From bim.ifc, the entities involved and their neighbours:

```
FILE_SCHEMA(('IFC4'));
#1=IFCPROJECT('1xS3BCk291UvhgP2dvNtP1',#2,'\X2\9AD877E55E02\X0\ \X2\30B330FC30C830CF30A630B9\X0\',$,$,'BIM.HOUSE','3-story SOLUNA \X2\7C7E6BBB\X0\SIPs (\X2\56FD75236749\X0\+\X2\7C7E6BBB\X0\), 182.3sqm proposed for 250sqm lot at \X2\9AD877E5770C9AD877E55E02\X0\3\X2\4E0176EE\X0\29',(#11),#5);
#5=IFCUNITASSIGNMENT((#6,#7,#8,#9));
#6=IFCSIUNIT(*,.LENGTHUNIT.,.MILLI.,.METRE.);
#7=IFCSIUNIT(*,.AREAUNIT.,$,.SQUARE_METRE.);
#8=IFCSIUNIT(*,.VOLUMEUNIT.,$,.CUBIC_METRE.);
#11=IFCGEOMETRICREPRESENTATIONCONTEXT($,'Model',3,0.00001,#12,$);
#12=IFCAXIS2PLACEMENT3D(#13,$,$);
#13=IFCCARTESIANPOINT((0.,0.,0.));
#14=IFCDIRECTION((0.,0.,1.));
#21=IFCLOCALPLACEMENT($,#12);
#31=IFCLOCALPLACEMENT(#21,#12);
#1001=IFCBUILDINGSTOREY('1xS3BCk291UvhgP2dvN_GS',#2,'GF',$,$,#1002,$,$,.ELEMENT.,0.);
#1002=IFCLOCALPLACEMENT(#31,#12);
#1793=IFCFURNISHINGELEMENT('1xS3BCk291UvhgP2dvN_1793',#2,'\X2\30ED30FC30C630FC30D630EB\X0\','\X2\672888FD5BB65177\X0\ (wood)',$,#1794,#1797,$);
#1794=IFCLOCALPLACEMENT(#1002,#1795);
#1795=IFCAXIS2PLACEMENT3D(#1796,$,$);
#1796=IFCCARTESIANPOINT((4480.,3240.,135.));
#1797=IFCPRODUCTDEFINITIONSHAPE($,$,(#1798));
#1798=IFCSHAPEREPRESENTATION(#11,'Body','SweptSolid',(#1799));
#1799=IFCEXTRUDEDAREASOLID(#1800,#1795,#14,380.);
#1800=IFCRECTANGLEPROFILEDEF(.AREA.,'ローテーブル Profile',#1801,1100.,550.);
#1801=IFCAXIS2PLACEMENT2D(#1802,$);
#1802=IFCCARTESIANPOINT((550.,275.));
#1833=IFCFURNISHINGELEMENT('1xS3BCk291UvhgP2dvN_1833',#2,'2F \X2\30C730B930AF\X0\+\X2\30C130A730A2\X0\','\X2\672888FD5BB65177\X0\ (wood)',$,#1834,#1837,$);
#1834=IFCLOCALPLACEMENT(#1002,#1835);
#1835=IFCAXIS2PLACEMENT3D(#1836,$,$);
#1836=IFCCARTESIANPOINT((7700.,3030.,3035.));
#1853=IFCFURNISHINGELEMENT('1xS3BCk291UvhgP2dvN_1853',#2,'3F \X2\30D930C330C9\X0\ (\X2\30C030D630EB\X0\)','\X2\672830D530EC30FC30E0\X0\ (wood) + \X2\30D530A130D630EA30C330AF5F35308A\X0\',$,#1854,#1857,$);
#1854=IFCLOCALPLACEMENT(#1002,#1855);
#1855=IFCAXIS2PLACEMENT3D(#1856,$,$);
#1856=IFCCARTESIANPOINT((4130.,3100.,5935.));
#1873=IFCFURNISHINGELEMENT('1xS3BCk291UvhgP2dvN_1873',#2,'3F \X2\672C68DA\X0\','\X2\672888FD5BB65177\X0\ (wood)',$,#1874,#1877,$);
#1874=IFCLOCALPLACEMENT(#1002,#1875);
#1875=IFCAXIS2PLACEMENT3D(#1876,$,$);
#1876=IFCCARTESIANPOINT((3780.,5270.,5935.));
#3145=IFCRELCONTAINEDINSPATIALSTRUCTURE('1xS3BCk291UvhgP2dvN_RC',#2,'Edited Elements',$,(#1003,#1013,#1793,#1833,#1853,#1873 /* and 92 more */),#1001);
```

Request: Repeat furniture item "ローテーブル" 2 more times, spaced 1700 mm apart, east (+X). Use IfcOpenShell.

```python
import numpy as np
import ifcopenshell
import ifcopenshell.api.geometry
import ifcopenshell.api.root
import ifcopenshell.util.element
import ifcopenshell.util.placement
import ifcopenshell.util.unit

model = ifcopenshell.open("bim.ifc")
unit_scale = ifcopenshell.util.unit.calculate_unit_scale(model)


def reuse_history(source, copy):
    """copy_class also copies each property set's owner history, people and application; keep the originals."""
    for rel in copy.IsDefinedBy:
        if rel.is_a("IfcRelDefinesByProperties") and (history := rel.RelatingPropertyDefinition.OwnerHistory):
            rel.RelatingPropertyDefinition.OwnerHistory = source.OwnerHistory
            ifcopenshell.util.element.remove_deep2(model, history)


source = model.by_guid("1xS3BCk291UvhgP2dvN_1793")
base = ifcopenshell.util.placement.get_local_placement(source.ObjectPlacement)
step = np.array([1.0, 0.0, 0.0]) * 1.7 / unit_scale

for i in range(1, 3):
    copy = ifcopenshell.api.root.copy_class(model, product=source)
    copy.Representation = ifcopenshell.util.element.copy_deep(
        model, source.Representation, exclude=["IfcGeometricRepresentationContext", "IfcRepresentationMap"]
    )
    reuse_history(source, copy)
    matrix = base.copy()
    matrix[:3, 3] += i * step
    print("added at", matrix[:3, 3].round(3) + 0.0)
    ifcopenshell.api.geometry.edit_object_placement(model, product=copy, matrix=matrix, is_si=False)

model.write("bim_updated.ifc")
```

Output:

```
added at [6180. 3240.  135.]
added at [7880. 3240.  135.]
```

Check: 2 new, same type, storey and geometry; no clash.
